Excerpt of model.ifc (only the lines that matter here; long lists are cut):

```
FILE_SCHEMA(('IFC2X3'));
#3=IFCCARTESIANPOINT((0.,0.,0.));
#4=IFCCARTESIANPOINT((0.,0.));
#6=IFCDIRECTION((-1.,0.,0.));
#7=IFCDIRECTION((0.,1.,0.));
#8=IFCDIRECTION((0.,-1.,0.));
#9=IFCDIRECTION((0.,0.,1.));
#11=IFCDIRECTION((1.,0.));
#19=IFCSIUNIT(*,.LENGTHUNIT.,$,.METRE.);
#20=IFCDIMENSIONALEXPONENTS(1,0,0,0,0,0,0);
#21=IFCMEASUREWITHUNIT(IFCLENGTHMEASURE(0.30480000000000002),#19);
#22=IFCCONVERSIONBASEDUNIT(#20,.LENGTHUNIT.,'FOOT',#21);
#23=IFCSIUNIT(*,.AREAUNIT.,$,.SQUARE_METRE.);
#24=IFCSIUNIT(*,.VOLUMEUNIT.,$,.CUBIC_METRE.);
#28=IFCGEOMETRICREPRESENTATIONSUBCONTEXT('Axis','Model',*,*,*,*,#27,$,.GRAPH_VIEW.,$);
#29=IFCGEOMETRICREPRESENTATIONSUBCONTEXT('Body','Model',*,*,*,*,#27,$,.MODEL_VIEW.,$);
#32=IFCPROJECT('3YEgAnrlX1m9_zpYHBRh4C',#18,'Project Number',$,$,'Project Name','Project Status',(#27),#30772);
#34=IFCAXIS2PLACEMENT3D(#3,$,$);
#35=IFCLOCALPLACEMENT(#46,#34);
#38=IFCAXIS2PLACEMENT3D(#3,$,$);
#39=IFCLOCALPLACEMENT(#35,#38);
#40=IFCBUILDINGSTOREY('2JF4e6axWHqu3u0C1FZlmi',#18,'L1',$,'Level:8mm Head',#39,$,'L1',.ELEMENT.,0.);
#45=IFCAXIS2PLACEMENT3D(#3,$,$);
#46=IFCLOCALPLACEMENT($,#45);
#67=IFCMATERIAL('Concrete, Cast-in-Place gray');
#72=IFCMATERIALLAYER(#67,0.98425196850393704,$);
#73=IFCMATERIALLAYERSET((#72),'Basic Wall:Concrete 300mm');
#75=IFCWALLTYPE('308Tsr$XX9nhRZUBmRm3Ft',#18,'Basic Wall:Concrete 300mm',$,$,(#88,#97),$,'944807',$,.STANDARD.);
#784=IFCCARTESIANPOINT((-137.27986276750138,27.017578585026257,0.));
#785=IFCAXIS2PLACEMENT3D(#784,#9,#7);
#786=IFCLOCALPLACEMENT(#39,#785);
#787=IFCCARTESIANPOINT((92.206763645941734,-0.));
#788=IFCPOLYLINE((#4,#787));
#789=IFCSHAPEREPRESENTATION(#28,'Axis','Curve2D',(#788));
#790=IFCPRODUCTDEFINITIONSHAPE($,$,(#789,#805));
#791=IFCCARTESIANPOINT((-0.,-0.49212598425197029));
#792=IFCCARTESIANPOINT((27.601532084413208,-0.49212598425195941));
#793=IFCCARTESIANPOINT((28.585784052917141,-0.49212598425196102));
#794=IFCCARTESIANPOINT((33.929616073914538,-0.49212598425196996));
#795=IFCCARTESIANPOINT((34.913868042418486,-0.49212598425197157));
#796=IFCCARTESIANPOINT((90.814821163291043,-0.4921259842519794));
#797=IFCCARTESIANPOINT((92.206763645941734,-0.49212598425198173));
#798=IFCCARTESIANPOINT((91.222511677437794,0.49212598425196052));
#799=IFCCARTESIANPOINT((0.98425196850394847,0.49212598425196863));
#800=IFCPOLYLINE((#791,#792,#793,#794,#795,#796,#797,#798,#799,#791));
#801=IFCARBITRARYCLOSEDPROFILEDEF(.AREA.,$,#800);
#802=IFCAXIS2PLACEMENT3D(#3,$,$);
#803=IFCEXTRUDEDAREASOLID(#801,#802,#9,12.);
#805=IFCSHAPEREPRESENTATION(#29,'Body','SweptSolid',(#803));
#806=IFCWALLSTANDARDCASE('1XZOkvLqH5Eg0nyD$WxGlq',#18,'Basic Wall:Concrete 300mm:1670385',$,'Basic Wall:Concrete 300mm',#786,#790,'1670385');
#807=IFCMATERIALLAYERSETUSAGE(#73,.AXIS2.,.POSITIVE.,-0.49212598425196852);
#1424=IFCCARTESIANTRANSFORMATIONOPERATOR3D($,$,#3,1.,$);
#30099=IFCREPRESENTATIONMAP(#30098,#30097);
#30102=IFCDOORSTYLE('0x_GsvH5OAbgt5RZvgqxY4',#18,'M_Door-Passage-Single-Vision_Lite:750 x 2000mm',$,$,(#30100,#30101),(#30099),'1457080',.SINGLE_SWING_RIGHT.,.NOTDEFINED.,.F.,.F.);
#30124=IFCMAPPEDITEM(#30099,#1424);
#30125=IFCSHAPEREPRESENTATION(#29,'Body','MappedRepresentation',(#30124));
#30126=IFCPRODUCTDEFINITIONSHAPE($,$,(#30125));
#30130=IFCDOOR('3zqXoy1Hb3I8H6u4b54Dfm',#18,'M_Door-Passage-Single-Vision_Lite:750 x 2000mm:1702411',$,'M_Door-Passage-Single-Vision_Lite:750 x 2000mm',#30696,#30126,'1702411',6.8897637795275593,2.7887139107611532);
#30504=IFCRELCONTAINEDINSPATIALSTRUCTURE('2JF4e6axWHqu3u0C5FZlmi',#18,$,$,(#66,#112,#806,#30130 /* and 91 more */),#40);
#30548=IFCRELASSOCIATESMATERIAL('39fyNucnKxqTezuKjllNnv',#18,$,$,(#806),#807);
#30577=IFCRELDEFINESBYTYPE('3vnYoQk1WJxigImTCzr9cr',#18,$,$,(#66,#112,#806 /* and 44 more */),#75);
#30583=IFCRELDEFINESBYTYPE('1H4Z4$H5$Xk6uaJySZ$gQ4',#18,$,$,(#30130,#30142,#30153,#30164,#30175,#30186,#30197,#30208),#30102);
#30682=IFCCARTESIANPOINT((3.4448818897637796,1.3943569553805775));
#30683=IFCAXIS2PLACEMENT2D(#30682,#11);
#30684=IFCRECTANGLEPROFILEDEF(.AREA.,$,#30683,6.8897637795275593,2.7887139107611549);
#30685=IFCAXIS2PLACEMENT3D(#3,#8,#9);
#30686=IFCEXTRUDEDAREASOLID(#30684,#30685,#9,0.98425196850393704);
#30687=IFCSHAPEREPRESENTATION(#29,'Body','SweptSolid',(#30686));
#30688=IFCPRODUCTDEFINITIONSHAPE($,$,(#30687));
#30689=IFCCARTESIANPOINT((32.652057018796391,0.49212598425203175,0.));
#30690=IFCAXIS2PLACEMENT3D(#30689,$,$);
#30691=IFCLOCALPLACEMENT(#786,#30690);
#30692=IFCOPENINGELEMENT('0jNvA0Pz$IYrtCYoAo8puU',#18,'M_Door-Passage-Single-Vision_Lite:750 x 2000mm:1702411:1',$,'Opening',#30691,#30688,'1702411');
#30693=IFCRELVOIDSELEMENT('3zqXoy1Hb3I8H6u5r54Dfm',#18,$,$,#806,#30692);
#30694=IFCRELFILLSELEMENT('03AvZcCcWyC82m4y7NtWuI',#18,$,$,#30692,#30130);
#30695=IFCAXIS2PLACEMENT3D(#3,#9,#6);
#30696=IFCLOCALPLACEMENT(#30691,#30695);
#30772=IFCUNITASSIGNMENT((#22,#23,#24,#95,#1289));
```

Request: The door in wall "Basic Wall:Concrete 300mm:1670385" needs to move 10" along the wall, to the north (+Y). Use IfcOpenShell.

```python
import ifcopenshell
import ifcopenshell.api.geometry
import ifcopenshell.util.placement
import ifcopenshell.util.unit

model = ifcopenshell.open("model.ifc")
unit_scale = ifcopenshell.util.unit.calculate_unit_scale(model)

door = model.by_guid("3zqXoy1Hb3I8H6u4b54Dfm")
opening = door.FillsVoids[0].RelatingOpeningElement
wall = opening.VoidsElements[0].RelatingBuildingElement

wall_matrix = ifcopenshell.util.placement.get_local_placement(wall.ObjectPlacement)
shift = wall_matrix[:3, 0] * 10 * 0.0254 / unit_scale
before = ifcopenshell.util.placement.get_local_placement(door.ObjectPlacement)[:3, 3].copy()

# The door is placed relative to its opening, so it follows when the opening moves.
matrix = ifcopenshell.util.placement.get_local_placement(opening.ObjectPlacement)
matrix[:3, 3] += shift
ifcopenshell.api.geometry.edit_object_placement(
    model, product=opening, matrix=matrix, is_si=False, should_transform_children=True
)

after = ifcopenshell.util.placement.get_local_placement(door.ObjectPlacement)[:3, 3]
print("door moved by", (after - before).round(3) + 0.0)

model.write("model_updated.ifc")
```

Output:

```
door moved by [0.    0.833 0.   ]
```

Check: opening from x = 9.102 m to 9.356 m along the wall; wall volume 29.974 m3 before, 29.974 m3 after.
